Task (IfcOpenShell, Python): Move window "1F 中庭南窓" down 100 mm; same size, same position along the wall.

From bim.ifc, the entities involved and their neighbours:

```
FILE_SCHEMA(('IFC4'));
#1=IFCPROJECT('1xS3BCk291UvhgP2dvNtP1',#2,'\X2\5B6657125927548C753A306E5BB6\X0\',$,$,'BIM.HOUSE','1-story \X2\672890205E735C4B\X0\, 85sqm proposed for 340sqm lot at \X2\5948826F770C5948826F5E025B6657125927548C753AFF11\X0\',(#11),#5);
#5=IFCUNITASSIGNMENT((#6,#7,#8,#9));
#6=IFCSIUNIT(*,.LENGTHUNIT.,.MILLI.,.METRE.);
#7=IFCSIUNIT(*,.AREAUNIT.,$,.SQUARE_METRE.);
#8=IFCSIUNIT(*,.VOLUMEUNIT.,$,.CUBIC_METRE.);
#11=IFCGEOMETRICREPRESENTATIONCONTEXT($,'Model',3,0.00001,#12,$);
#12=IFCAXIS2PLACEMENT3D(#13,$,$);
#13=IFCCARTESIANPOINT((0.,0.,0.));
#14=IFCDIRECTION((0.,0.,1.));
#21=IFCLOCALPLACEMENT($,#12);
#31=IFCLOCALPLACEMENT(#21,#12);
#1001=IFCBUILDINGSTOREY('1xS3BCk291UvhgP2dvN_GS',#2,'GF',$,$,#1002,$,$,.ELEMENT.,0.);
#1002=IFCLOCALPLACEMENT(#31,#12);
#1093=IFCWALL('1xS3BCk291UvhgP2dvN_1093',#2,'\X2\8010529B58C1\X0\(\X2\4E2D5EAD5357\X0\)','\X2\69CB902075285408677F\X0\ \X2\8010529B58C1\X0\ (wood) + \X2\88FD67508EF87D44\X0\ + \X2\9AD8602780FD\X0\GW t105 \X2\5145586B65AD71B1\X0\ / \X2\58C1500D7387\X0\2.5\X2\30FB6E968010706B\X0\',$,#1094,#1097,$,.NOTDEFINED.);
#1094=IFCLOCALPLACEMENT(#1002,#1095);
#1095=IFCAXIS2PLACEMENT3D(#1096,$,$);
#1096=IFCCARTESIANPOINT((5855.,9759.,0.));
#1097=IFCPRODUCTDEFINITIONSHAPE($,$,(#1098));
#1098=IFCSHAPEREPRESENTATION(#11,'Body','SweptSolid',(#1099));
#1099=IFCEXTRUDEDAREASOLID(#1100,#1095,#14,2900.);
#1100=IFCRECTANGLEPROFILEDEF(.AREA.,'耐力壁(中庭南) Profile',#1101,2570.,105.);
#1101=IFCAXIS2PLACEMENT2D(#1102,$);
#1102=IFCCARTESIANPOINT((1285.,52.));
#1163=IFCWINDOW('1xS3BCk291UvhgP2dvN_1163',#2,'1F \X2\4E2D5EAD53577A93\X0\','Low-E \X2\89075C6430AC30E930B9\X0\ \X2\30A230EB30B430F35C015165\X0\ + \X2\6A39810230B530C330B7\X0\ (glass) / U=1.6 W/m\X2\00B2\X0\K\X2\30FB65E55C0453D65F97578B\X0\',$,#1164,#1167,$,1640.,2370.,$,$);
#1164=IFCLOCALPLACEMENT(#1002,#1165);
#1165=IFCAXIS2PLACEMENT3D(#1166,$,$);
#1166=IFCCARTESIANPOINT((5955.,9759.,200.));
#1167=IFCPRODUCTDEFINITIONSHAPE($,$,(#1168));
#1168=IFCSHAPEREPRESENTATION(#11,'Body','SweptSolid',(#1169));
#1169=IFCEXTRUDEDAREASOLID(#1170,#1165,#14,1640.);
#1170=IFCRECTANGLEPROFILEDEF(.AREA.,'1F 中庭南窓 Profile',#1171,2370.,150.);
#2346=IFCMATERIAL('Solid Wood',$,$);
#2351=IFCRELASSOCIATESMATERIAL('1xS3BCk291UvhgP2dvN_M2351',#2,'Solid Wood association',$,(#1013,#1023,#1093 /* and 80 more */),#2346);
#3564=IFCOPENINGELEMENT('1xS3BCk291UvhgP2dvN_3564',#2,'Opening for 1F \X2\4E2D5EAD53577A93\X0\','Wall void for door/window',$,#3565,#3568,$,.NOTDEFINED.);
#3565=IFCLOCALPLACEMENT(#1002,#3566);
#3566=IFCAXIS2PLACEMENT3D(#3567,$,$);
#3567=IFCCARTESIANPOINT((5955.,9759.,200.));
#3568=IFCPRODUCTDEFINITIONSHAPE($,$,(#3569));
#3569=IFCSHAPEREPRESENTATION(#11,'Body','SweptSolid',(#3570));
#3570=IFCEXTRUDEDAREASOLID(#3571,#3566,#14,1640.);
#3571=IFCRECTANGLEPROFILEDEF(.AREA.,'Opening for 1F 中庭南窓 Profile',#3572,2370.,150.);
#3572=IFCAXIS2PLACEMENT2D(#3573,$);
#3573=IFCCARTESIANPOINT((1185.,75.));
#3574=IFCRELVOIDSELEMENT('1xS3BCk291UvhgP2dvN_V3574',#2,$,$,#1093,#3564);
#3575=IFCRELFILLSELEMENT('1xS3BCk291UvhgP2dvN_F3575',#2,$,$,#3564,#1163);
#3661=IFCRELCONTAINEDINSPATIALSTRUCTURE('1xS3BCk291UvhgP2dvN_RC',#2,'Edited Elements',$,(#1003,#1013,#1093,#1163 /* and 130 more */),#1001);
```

```python
import numpy as np
import ifcopenshell
import ifcopenshell.api.geometry
import ifcopenshell.util.placement
import ifcopenshell.util.unit

model = ifcopenshell.open("bim.ifc")
unit_scale = ifcopenshell.util.unit.calculate_unit_scale(model)

window = model.by_guid("1xS3BCk291UvhgP2dvN_1163")
opening = window.FillsVoids[0].RelatingOpeningElement
dz = -100.0

shift = np.array([0.0, 0.0, dz])
# The window is not placed relative to its opening, so move both.
for product in (opening, window):
    matrix = ifcopenshell.util.placement.get_local_placement(product.ObjectPlacement)
    matrix[:3, 3] += shift
    ifcopenshell.api.geometry.edit_object_placement(model, product=product, matrix=matrix, is_si=False)

print(f"moved by {dz * unit_scale:+.3f} m")

model.write("bim_v2.ifc")
```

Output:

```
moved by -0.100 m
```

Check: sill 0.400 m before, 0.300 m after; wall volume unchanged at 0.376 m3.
